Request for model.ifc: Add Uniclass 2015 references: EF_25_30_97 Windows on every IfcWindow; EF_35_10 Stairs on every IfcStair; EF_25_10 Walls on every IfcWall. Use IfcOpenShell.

First a look at what the model holds.

```python
import ifcopenshell

model = ifcopenshell.open("model.ifc")
print(model.schema)
print("classifications:", [c.Name for c in model.by_type("IfcClassification")])
for ifc_class in ("IfcDoor", "IfcRoof", "IfcStair", "IfcWall", "IfcWindow"):
    print(ifc_class, len(model.by_type(ifc_class)))
```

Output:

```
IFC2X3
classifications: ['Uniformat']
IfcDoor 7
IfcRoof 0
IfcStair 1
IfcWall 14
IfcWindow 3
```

```python
import ifcopenshell
import ifcopenshell.api.classification

model = ifcopenshell.open("model.ifc")

# IFC2X3 requires Source and Edition and has no link from the project to the system.
system = model.create_entity("IfcClassification", Source="NBS", Edition="2015", Name="Uniclass 2015")

codes = {
    "IfcWindow": ("EF_25_30_97", "Windows"),
    "IfcStair": ("EF_35_10", "Stairs"),
    "IfcWall": ("EF_25_10", "Walls"),
}
for ifc_class, (code, name) in codes.items():
    products = model.by_type(ifc_class)
    ifcopenshell.api.classification.add_reference(
        model, products=products, classification=system, identification=code, name=name
    )
    print(code, len(products))

model.write("model_rev.ifc")
```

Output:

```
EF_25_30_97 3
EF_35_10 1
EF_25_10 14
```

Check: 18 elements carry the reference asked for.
